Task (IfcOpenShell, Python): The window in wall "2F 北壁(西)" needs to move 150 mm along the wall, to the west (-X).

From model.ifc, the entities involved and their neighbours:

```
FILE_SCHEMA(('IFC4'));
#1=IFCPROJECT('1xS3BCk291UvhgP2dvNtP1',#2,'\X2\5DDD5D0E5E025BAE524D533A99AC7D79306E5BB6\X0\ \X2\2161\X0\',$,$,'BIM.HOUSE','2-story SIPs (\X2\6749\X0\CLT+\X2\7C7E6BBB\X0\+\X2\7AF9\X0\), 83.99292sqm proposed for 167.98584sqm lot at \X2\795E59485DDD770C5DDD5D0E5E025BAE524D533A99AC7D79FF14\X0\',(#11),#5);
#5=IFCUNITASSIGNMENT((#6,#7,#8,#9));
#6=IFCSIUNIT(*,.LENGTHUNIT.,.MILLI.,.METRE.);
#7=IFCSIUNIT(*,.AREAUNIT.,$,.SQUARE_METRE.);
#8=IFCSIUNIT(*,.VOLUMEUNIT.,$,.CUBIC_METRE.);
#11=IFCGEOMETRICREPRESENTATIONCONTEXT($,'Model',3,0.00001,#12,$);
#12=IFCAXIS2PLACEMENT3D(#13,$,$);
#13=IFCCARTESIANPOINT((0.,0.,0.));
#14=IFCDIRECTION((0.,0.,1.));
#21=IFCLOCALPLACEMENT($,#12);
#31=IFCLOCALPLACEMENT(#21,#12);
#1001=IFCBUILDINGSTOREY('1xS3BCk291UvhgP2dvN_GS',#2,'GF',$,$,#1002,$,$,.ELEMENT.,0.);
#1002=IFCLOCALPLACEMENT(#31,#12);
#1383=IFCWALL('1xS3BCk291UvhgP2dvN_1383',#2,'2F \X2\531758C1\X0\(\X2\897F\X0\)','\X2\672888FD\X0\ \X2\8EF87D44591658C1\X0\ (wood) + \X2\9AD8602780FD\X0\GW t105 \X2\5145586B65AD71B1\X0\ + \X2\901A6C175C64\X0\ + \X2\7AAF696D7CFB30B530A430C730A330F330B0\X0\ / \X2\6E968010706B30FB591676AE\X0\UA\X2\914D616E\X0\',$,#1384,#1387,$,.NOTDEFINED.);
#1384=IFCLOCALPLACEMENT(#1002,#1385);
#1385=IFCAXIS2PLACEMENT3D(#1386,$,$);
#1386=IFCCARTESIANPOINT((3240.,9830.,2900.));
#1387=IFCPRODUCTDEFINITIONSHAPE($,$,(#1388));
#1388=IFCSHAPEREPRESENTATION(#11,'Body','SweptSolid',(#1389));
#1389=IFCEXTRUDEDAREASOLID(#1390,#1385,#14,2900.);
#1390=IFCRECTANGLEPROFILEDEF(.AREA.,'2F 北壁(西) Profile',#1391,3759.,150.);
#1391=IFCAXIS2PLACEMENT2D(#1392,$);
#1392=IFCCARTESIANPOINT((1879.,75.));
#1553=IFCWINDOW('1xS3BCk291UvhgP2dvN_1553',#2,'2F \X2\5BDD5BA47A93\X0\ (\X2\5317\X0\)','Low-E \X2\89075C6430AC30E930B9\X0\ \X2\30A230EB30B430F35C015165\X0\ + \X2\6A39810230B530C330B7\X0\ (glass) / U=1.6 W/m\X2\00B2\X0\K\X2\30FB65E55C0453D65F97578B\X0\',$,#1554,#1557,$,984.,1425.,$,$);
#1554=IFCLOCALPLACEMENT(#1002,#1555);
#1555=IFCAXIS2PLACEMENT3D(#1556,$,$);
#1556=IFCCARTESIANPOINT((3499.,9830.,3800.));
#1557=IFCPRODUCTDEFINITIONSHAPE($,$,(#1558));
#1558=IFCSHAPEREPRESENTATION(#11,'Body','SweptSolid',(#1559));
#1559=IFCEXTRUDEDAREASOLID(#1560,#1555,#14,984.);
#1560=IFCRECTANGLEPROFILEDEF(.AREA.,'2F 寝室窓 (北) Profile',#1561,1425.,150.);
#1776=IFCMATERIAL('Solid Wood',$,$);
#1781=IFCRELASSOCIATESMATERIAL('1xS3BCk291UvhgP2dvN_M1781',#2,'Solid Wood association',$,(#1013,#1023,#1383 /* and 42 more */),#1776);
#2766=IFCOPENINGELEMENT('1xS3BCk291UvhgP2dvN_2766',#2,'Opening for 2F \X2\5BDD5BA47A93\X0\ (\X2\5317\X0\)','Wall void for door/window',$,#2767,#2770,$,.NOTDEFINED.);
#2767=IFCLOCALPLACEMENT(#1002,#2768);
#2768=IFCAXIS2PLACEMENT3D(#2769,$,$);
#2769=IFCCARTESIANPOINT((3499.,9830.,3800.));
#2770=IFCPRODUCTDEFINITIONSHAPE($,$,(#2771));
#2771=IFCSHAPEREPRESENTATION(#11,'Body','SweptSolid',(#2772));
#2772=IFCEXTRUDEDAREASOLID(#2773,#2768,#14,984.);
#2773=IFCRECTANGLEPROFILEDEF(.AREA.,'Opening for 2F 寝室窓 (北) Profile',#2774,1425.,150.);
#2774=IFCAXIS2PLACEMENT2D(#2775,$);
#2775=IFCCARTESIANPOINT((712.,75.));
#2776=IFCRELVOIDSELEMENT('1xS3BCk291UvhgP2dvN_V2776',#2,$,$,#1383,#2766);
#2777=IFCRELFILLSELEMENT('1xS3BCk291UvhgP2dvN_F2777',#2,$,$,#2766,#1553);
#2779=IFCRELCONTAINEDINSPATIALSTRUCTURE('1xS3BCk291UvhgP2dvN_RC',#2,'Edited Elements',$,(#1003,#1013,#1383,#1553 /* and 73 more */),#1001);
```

```python
import ifcopenshell
import ifcopenshell.api.geometry
import ifcopenshell.util.placement

model = ifcopenshell.open("model.ifc")

window = model.by_guid("1xS3BCk291UvhgP2dvN_1553")
opening = window.FillsVoids[0].RelatingOpeningElement
wall = opening.VoidsElements[0].RelatingBuildingElement

wall_matrix = ifcopenshell.util.placement.get_local_placement(wall.ObjectPlacement)
shift = wall_matrix[:3, 0] * -150.0
before = ifcopenshell.util.placement.get_local_placement(window.ObjectPlacement)[:3, 3].copy()

# The window is not placed relative to its opening, so move both.
for product in (opening, window):
    matrix = ifcopenshell.util.placement.get_local_placement(product.ObjectPlacement)
    matrix[:3, 3] += shift
    ifcopenshell.api.geometry.edit_object_placement(model, product=product, matrix=matrix, is_si=False)

after = ifcopenshell.util.placement.get_local_placement(window.ObjectPlacement)[:3, 3]
print("window moved by", (after - before).round(3) + 0.0)

model.write("model-out.ifc")
```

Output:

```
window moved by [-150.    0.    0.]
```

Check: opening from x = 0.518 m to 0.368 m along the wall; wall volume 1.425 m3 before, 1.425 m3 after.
